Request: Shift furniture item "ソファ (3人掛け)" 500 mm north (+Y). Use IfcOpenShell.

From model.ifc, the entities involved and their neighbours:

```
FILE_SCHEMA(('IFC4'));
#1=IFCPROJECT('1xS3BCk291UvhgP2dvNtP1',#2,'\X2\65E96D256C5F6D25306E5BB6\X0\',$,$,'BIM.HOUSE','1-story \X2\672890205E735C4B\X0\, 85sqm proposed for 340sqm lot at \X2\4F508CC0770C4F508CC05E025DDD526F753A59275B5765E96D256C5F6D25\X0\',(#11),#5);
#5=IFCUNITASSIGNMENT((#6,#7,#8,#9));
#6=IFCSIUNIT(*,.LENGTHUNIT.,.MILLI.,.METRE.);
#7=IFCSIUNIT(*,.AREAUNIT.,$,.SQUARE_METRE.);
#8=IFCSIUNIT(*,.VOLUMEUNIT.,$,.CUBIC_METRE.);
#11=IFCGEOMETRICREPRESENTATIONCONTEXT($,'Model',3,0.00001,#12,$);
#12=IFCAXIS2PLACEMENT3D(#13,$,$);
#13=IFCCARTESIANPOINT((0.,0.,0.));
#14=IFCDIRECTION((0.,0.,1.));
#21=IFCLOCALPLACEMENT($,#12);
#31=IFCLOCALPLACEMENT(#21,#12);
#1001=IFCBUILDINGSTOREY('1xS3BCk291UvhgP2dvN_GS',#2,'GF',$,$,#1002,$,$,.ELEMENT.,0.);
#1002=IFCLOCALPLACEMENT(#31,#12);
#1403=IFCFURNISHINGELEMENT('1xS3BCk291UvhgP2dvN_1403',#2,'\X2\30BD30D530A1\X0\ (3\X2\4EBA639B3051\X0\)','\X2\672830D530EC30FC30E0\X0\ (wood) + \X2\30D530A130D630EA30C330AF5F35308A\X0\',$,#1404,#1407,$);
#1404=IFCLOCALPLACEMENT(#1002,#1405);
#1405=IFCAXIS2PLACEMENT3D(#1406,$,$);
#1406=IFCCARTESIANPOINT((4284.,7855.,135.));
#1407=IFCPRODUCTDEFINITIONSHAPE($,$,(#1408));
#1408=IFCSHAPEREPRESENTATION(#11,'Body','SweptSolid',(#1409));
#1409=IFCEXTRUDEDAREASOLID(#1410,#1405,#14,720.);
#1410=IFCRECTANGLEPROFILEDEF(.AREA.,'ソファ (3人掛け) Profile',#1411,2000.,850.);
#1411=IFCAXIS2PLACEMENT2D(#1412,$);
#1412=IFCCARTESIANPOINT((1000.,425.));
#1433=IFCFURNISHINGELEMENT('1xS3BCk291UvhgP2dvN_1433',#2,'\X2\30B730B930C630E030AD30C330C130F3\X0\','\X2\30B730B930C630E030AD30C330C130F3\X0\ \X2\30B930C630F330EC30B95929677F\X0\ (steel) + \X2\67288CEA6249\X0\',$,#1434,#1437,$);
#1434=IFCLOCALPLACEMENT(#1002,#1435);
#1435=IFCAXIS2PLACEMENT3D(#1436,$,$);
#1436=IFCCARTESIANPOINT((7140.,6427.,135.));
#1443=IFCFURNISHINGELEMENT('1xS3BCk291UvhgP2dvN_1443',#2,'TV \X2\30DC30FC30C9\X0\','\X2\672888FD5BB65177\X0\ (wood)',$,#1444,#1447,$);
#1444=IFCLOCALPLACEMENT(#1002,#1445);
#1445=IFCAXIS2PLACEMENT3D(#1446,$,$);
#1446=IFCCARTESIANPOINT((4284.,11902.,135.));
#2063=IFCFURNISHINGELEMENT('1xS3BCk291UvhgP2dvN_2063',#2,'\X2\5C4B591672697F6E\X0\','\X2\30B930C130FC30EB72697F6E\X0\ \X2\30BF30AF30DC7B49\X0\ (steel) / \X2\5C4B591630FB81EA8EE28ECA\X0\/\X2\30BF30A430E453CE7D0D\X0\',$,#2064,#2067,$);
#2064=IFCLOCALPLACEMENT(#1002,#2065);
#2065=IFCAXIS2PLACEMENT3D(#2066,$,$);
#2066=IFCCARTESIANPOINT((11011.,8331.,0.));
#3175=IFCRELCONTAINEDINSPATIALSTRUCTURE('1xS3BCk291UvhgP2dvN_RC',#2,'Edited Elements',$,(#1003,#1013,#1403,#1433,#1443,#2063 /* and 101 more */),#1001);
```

```python
import ifcopenshell
import ifcopenshell.api.geometry
import ifcopenshell.util.placement
import ifcopenshell.util.unit

model = ifcopenshell.open("model.ifc")
unit_scale = ifcopenshell.util.unit.calculate_unit_scale(model)

item = model.by_id(1403)
matrix = ifcopenshell.util.placement.get_local_placement(item.ObjectPlacement)
matrix[1, 3] += 0.5 / unit_scale
ifcopenshell.api.geometry.edit_object_placement(model, product=item, matrix=matrix, is_si=False)

print(ifcopenshell.util.placement.get_local_placement(item.ObjectPlacement).round(3) + 0.0)

model.write("model-out.ifc")
```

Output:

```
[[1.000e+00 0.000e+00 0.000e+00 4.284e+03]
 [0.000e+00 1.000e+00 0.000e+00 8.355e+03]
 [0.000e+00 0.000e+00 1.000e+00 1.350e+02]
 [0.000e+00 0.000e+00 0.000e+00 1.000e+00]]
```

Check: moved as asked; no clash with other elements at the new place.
